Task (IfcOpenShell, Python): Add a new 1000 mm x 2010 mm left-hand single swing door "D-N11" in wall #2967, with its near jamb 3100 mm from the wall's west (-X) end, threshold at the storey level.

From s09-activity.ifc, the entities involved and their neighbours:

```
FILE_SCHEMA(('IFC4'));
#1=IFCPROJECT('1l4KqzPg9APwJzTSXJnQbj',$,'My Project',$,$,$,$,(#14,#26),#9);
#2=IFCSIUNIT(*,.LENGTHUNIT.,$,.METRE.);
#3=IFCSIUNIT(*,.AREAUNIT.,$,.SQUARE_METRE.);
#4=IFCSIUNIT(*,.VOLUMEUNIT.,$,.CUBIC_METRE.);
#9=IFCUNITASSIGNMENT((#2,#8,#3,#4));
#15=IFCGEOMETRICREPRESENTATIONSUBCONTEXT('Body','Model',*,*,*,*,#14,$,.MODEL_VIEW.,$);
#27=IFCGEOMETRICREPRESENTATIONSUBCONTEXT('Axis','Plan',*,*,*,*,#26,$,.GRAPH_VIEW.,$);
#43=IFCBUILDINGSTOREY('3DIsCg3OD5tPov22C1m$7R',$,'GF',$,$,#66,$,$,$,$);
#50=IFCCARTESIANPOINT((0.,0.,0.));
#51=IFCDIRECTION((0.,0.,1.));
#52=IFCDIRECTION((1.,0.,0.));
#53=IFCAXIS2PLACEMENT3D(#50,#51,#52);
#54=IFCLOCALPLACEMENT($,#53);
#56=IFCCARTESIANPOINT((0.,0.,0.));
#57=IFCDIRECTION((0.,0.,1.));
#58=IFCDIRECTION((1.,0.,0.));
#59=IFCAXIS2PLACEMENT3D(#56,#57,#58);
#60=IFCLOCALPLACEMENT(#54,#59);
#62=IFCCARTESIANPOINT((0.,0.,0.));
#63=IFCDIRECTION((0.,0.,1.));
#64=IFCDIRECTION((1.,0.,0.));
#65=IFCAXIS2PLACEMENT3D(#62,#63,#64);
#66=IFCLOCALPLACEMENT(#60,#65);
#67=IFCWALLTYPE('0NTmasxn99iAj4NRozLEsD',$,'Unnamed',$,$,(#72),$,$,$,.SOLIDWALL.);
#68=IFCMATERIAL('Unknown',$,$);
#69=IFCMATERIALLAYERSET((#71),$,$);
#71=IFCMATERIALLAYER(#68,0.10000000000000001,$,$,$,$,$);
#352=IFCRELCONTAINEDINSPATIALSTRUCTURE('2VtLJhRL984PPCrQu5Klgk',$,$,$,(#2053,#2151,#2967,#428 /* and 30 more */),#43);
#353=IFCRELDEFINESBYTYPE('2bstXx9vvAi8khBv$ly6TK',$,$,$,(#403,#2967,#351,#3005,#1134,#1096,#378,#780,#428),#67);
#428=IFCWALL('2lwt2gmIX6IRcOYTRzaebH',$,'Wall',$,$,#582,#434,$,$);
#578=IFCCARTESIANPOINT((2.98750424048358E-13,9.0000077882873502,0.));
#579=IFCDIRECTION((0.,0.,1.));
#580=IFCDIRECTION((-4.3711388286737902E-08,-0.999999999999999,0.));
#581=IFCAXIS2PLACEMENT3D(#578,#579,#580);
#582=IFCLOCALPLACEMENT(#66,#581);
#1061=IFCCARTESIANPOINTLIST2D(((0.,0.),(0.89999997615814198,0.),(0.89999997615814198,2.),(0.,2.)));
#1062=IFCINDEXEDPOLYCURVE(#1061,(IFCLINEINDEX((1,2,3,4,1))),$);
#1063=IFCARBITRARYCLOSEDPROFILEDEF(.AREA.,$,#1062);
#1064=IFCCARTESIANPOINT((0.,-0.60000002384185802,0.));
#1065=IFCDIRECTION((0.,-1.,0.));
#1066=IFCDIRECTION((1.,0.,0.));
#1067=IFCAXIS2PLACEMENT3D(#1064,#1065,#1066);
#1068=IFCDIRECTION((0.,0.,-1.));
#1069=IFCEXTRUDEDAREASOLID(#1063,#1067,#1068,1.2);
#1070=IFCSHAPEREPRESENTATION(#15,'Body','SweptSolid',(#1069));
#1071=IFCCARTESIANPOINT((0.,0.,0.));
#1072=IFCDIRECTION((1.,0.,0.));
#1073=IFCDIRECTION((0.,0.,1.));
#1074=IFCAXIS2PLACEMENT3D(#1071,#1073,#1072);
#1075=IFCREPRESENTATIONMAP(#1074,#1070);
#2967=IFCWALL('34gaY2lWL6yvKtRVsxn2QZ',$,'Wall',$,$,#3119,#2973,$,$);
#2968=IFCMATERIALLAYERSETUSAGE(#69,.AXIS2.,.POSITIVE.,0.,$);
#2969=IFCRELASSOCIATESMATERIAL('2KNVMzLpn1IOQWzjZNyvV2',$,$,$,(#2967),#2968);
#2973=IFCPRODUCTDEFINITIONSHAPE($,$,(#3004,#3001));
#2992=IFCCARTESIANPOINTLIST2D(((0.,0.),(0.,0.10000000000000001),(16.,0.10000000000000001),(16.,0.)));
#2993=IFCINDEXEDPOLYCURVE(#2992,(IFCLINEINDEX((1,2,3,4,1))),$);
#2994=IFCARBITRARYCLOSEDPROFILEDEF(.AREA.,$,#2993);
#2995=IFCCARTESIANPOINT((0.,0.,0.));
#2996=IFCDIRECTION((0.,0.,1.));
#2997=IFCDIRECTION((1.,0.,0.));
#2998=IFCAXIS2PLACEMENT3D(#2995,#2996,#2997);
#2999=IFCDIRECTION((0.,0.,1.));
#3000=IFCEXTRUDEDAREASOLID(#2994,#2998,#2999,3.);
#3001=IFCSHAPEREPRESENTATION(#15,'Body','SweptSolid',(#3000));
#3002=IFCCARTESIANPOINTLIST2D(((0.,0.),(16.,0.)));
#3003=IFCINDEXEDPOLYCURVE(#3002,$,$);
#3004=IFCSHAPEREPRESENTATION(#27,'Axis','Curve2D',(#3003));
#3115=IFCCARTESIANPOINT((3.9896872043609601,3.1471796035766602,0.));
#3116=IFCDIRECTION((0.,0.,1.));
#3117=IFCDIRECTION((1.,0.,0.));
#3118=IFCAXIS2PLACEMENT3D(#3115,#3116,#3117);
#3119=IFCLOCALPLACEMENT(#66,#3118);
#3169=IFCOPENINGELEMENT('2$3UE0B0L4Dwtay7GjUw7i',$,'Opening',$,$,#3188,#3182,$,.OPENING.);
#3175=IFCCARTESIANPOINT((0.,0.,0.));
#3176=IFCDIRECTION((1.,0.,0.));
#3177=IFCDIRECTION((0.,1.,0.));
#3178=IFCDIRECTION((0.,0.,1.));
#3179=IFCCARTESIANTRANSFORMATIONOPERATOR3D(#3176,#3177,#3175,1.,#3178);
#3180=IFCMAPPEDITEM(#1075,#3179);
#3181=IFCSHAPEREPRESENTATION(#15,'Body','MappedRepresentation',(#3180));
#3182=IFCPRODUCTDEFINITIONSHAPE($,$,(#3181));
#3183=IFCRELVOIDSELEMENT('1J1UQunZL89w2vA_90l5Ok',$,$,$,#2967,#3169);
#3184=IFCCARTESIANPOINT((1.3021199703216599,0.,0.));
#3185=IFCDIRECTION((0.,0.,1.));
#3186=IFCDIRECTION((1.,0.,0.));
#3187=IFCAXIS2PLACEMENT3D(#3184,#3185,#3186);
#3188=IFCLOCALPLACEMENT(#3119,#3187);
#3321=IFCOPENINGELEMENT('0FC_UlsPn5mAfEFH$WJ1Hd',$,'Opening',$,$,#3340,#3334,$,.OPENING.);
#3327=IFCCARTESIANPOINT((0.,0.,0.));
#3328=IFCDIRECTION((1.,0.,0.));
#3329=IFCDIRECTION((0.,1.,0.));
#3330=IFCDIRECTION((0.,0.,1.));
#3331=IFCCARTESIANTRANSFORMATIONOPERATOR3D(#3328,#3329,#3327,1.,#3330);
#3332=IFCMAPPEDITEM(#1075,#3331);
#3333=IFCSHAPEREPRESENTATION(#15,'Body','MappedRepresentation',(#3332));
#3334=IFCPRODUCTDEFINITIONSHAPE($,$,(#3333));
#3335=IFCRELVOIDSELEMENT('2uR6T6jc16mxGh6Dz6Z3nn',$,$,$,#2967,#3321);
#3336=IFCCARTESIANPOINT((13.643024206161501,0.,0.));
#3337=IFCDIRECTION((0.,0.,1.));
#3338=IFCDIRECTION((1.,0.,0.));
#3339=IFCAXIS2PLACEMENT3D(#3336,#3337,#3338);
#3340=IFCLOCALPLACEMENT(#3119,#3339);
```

```python
import numpy as np
import ifcopenshell
import ifcopenshell.api.feature
import ifcopenshell.api.geometry
import ifcopenshell.api.root
import ifcopenshell.api.spatial
import ifcopenshell.geom
import ifcopenshell.util.element
import ifcopenshell.util.placement
import ifcopenshell.util.representation
import ifcopenshell.util.shape
import ifcopenshell.util.unit

model = ifcopenshell.open("s09-activity.ifc")
unit_scale = ifcopenshell.util.unit.calculate_unit_scale(model)
settings = ifcopenshell.geom.settings()


def volume(element):
    """Net volume in cubic metres, openings subtracted."""
    shape = ifcopenshell.geom.create_shape(settings, element)
    return ifcopenshell.util.shape.get_volume(shape.geometry)


wall = model.by_guid("34gaY2lWL6yvKtRVsxn2QZ")
storey = ifcopenshell.util.element.get_container(wall, ifc_class="IfcBuildingStorey")
context = ifcopenshell.util.representation.get_context(model, "Model", "Body", "MODEL_VIEW")
before = volume(wall)

width, height, from_end, sill = 1, 2.01, 3.1, 0.0  # metres

# The wall runs along its own X axis, and the end named is its -X end.
wall_shape = ifcopenshell.geom.create_shape(settings, wall)
x, y, z = ifcopenshell.util.shape.get_vertices(wall_shape.geometry).T
start = x.min() + from_end
face, thickness = float(y.min()), float(y.max() - y.min())
wall_matrix = ifcopenshell.util.placement.get_local_placement(wall.ObjectPlacement)
level = ifcopenshell.util.placement.get_local_placement(storey.ObjectPlacement)[2, 3]


def in_wall(x, y):
    """Placement at x, y metres in the wall's axes, at sill height."""
    matrix = wall_matrix.copy()
    matrix[:, 3] = wall_matrix @ np.array([x / unit_scale, y / unit_scale, 0.0, 1.0])
    matrix[2, 3] = level + sill / unit_scale
    return matrix


# Opening: a box that overshoots both wall faces by 50 mm.
opening = ifcopenshell.api.root.create_entity(model, ifc_class="IfcOpeningElement", predefined_type="OPENING")
box = ifcopenshell.api.geometry.add_wall_representation(
    model, context=context, length=width, height=height, thickness=thickness + 0.1
)
ifcopenshell.api.geometry.assign_representation(model, product=opening, representation=box)
ifcopenshell.api.geometry.edit_object_placement(model, product=opening, matrix=in_wall(start, face - 0.05), is_si=False)
ifcopenshell.api.feature.add_feature(model, feature=opening, element=wall)

door = ifcopenshell.api.root.create_entity(model, ifc_class="IfcDoor", name="D-N11", predefined_type="DOOR")
door.OverallWidth, door.OverallHeight = width / unit_scale, height / unit_scale
door.OperationType = "SINGLE_SWING_LEFT"
body = ifcopenshell.api.geometry.add_door_representation(
    model,
    context=context,
    overall_width=door.OverallWidth,
    overall_height=door.OverallHeight,
    operation_type="SINGLE_SWING_LEFT",
    lining_properties={"LiningDepth": thickness / unit_scale, "ThresholdDepth": thickness / unit_scale},
)
ifcopenshell.api.geometry.assign_representation(model, product=door, representation=body)
ifcopenshell.api.spatial.assign_container(model, products=[door], relating_structure=storey)
ifcopenshell.api.feature.add_filling(model, opening=opening, element=door)

# The lining spans the wall, so the door starts at the wall face.
ifcopenshell.api.geometry.edit_object_placement(model, product=door, matrix=in_wall(start, face), is_si=False)

after = volume(wall)

print(f"wall volume {before:.3f} -> {after:.3f} m3")

model.write("s09-activity_updated.ifc")
```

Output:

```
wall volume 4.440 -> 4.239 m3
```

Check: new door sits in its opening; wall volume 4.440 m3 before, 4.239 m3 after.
